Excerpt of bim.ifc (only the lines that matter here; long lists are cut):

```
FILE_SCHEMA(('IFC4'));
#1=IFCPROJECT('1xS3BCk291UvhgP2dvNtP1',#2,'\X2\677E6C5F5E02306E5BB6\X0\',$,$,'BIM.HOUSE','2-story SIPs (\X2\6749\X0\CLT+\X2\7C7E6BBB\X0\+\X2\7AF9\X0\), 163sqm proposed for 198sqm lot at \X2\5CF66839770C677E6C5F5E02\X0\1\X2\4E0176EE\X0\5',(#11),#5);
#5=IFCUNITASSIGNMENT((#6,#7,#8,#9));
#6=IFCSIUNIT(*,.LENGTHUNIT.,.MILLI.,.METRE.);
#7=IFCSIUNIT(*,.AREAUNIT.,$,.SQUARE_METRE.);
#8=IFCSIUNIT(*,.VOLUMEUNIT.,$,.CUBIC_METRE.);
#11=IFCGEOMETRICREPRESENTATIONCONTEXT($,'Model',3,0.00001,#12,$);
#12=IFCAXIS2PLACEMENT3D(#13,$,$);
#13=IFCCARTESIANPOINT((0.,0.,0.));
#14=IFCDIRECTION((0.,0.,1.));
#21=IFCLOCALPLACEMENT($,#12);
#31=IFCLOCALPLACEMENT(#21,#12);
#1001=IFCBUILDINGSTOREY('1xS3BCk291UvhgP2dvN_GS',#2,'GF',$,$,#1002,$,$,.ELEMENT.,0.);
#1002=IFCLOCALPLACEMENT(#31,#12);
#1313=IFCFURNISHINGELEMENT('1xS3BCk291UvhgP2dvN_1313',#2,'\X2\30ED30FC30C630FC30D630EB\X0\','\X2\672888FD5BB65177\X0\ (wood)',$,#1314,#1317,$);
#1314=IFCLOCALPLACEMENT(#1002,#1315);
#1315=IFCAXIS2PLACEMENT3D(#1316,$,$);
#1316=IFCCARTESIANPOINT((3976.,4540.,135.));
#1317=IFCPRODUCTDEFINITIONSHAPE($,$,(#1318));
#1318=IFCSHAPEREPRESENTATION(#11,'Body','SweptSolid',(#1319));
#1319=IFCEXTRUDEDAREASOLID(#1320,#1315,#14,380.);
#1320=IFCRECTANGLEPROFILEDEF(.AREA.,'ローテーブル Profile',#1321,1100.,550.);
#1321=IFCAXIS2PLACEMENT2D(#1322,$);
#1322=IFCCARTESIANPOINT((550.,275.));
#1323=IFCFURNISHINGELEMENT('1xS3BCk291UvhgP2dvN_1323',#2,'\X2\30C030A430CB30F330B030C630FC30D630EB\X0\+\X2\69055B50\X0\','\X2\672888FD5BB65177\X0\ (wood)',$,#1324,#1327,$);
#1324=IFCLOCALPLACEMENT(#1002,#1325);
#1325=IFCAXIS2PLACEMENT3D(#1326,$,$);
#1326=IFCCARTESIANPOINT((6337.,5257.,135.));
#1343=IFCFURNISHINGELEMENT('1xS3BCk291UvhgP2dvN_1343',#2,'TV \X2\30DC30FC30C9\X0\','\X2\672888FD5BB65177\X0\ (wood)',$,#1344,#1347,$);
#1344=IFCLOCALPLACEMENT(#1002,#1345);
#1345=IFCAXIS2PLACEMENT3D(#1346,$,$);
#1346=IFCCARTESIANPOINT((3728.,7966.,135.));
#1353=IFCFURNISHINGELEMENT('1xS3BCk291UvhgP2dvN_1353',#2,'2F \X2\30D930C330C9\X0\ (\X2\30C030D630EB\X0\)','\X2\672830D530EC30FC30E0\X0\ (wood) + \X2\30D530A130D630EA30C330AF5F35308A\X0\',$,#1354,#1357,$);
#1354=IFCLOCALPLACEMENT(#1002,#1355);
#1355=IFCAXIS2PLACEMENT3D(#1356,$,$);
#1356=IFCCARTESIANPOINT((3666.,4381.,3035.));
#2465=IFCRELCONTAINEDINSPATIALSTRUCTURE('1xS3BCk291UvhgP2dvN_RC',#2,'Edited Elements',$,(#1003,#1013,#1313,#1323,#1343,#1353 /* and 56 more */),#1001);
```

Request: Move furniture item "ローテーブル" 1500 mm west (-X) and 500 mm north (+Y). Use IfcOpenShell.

```python
import ifcopenshell
import ifcopenshell.api.geometry
import ifcopenshell.util.placement
import ifcopenshell.util.unit

model = ifcopenshell.open("bim.ifc")
unit_scale = ifcopenshell.util.unit.calculate_unit_scale(model)

item = model.by_id(1313)
matrix = ifcopenshell.util.placement.get_local_placement(item.ObjectPlacement)
matrix[0, 3] -= 1.5 / unit_scale
matrix[1, 3] += 0.5 / unit_scale
ifcopenshell.api.geometry.edit_object_placement(model, product=item, matrix=matrix, is_si=False)

print(ifcopenshell.util.placement.get_local_placement(item.ObjectPlacement).round(3) + 0.0)

model.write("bim_rev.ifc")
```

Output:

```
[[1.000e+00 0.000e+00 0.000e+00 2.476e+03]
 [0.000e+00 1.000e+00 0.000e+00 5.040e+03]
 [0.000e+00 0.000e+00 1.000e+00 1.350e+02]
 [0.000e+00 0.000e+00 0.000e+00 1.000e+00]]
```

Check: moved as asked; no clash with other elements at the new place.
